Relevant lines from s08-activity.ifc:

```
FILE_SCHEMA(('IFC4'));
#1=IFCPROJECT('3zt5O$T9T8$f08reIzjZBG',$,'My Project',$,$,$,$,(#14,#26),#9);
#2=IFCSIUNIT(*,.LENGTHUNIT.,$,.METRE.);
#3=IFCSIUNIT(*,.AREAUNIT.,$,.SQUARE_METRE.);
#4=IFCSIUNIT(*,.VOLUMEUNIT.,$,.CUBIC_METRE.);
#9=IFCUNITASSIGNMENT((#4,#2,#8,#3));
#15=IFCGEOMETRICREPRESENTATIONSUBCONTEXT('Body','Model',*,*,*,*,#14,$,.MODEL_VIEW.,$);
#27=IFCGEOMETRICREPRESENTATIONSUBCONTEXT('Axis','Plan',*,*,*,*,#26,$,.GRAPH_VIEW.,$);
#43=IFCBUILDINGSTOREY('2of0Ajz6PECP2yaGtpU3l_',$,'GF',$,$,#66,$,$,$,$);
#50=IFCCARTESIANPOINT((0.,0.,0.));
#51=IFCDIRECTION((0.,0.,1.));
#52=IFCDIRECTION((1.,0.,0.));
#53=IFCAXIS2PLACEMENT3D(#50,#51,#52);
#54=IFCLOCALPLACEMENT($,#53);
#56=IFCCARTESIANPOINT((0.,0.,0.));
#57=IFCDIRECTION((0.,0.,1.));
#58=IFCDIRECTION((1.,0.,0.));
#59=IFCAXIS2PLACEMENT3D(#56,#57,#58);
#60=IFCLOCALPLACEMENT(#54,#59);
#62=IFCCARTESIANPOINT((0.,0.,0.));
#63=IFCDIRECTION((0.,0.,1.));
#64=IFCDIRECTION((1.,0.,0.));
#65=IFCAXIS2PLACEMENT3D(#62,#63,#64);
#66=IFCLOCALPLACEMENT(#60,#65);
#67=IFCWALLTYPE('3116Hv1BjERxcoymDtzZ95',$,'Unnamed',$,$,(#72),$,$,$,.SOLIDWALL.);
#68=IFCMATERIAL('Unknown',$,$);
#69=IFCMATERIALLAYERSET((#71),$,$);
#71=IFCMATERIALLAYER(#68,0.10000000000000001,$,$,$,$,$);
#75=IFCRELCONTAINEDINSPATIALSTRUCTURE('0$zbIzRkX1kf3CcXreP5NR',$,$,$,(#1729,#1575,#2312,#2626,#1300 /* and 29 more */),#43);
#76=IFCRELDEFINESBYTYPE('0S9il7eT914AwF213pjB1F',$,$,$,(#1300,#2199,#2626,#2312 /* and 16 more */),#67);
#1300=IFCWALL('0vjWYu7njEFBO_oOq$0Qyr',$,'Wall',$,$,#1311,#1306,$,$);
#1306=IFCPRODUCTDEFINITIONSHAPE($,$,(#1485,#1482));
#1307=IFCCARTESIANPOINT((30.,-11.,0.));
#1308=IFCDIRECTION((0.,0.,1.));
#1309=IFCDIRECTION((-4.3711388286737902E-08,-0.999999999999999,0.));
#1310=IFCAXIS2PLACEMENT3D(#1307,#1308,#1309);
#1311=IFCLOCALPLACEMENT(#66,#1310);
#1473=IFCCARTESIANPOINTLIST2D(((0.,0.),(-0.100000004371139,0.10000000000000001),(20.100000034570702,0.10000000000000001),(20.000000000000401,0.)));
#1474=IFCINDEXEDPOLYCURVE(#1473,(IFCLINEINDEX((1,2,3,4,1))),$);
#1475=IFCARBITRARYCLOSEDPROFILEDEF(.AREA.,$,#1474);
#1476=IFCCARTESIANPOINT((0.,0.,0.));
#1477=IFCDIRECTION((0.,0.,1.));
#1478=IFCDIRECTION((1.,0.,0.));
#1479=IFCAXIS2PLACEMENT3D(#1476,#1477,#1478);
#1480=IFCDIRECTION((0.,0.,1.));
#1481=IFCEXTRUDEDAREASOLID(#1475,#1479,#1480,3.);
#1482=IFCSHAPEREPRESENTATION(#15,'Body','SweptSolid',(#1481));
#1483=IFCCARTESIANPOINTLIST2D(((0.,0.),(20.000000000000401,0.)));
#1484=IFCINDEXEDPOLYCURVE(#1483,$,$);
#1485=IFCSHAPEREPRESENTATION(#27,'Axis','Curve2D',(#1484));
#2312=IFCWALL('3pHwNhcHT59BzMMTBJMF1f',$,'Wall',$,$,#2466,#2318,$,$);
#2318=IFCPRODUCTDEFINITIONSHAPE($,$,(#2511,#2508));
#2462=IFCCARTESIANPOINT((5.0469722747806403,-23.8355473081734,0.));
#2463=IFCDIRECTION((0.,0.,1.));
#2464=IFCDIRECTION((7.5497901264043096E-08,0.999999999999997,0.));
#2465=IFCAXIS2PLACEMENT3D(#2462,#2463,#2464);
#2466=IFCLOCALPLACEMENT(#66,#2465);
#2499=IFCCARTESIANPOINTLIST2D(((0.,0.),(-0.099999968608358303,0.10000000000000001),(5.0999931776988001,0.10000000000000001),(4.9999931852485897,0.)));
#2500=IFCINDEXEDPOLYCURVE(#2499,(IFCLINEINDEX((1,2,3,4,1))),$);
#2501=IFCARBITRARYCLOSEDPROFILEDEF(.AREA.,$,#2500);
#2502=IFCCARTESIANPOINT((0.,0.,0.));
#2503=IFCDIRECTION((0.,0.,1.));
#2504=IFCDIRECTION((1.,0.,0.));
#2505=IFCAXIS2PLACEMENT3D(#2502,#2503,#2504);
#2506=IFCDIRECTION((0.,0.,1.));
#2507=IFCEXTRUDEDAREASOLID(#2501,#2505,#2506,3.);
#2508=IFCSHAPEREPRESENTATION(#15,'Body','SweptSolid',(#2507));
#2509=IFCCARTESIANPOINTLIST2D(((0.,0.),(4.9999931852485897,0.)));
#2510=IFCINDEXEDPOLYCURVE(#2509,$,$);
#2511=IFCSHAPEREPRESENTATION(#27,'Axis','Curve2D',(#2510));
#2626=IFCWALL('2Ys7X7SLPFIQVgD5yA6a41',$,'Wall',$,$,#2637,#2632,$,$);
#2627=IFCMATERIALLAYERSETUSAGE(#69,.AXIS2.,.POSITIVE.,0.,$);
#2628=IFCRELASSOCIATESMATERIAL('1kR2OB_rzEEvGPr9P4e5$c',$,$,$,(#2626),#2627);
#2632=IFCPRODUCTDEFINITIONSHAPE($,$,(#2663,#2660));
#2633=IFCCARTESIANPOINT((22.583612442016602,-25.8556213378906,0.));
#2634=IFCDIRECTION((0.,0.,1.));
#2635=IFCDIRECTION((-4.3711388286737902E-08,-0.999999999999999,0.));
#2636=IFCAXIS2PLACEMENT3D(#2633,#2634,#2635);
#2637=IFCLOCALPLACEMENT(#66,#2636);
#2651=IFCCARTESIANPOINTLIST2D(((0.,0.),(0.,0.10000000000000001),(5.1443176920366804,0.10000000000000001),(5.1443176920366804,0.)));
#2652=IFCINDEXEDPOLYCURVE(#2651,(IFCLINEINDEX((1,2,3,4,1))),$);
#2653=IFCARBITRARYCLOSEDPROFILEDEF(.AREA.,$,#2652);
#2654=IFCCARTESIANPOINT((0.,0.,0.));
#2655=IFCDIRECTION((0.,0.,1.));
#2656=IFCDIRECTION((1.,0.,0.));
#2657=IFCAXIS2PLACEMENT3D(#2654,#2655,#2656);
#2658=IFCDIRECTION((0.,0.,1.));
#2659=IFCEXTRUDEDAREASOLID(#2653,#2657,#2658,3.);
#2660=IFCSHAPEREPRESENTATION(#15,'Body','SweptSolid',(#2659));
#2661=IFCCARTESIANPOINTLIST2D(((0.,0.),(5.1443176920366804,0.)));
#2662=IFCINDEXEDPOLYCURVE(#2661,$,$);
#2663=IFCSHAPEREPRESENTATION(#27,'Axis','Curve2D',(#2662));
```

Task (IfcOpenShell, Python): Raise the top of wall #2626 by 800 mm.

```python
import ifcopenshell
import ifcopenshell.geom
import ifcopenshell.util.representation
import ifcopenshell.util.shape
import ifcopenshell.util.unit

model = ifcopenshell.open("s08-activity.ifc")
unit_scale = ifcopenshell.util.unit.calculate_unit_scale(model)
settings = ifcopenshell.geom.settings()


def volume(element):
    """Net volume in cubic metres, openings subtracted."""
    shape = ifcopenshell.geom.create_shape(settings, element)
    return ifcopenshell.util.shape.get_volume(shape.geometry)


wall = model.by_guid("2Ys7X7SLPFIQVgD5yA6a41")
before = volume(wall)

body = ifcopenshell.util.representation.get_representation(wall, "Model", "Body")
solid = body.Items[0]
old_height = solid.Depth
solid.Depth += 0.8 / unit_scale
after = volume(wall)

print(f"height {old_height:g} -> {solid.Depth:g}, volume {before:.3f} -> {after:.3f} m3")

model.write("s08-activity_v2.ifc")
```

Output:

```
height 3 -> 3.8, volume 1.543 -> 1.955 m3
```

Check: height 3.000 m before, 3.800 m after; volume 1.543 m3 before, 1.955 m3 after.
